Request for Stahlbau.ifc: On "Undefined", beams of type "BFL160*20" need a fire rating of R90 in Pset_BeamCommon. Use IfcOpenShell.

First a look at what the model holds.

```python
import ifcopenshell
import ifcopenshell.util.element

model = ifcopenshell.open("Stahlbau.ifc")
print(model.schema)
storey = next(s for s in model.by_type("IfcBuildingStorey") if s.Name == "Undefined")
beams = [e for e in ifcopenshell.util.element.get_decomposition(storey) if e.is_a("IfcBeam")]
seen = {}
for e in beams:
    element_type = ifcopenshell.util.element.get_type(e)
    key = (element_type.Name if element_type != e and element_type else None, ifcopenshell.util.element.get_pset(e, "Pset_BeamCommon", "FireRating"))
    seen[key] = seen.get(key, 0) + 1
for (name, value), count in sorted(seen.items(), key=str):
    print(count, "x", name, "|", value)
```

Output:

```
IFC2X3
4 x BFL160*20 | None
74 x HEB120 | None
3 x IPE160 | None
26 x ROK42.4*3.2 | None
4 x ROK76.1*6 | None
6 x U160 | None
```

```python
import ifcopenshell
import ifcopenshell.api.pset
import ifcopenshell.util.element

model = ifcopenshell.open("Stahlbau.ifc")

storey = next(s for s in model.by_type("IfcBuildingStorey") if s.Name == "Undefined")
beams = [e for e in ifcopenshell.util.element.get_decomposition(storey) if e.is_a("IfcBeam")]

count = 0
for e in beams:
    element_type = ifcopenshell.util.element.get_type(e)
    if element_type in (None, e) or element_type.Name != "BFL160*20":
        continue
    # add_pset returns the element's existing set when there is one.
    pset = ifcopenshell.api.pset.add_pset(model, product=e, name="Pset_BeamCommon")
    ifcopenshell.api.pset.edit_pset(model, pset=pset, properties={"FireRating": "R90"})
    count += 1

print(count, "beams updated")

model.write("Stahlbau_updated.ifc")
```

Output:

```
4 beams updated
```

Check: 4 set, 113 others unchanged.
